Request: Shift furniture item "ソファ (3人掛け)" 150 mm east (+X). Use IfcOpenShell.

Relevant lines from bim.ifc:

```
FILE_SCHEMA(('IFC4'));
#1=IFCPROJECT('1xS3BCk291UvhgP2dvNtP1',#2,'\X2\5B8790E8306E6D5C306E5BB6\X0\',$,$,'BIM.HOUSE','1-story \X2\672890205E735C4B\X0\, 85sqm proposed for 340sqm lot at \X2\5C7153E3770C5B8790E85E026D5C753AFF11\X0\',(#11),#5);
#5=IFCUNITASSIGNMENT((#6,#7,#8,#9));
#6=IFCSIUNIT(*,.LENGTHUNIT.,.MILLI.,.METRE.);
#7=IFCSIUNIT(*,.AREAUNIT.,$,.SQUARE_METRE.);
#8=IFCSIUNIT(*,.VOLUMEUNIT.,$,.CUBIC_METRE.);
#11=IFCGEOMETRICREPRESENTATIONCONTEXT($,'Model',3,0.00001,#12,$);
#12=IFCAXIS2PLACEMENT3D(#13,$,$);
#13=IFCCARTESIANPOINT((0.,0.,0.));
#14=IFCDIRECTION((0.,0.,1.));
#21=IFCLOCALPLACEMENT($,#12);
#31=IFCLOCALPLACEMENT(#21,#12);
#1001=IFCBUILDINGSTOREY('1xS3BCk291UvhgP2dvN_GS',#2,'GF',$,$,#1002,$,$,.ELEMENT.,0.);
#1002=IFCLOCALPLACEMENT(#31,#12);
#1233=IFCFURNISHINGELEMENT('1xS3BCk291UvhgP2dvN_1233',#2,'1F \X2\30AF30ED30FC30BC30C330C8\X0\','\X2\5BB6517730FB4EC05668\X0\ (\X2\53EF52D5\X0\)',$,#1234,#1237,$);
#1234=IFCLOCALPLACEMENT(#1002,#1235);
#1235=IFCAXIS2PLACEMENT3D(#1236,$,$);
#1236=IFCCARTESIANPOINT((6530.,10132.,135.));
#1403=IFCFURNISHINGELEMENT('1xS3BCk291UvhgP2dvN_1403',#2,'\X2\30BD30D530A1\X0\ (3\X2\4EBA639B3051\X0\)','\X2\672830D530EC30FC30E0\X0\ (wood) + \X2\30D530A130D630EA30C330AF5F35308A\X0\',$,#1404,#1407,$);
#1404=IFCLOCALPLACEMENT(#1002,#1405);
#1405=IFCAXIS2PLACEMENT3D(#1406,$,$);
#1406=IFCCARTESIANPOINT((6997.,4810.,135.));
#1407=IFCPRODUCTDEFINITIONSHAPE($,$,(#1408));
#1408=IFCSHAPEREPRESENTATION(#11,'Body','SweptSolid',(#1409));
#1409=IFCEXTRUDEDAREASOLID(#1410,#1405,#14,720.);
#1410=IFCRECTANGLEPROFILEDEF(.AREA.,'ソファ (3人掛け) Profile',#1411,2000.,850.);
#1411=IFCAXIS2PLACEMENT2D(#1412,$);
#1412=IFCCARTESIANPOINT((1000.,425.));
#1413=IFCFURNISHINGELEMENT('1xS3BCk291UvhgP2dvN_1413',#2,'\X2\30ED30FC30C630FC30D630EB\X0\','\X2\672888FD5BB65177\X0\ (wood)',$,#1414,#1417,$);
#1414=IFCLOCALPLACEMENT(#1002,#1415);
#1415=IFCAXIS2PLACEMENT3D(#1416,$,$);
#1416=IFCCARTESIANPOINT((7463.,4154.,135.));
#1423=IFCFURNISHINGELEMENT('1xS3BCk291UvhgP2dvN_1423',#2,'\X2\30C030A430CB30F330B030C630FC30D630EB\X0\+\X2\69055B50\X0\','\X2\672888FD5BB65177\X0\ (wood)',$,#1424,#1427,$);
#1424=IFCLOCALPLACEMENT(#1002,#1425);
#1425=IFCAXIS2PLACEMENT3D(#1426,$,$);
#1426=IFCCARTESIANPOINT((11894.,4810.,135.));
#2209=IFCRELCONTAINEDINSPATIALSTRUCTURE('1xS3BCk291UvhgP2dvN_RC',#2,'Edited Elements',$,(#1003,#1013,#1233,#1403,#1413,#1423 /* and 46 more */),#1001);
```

```python
import ifcopenshell
import ifcopenshell.api.geometry
import ifcopenshell.util.placement
import ifcopenshell.util.unit

model = ifcopenshell.open("bim.ifc")
unit_scale = ifcopenshell.util.unit.calculate_unit_scale(model)

item = model.by_id(1403)
matrix = ifcopenshell.util.placement.get_local_placement(item.ObjectPlacement)
matrix[0, 3] += 0.15 / unit_scale
ifcopenshell.api.geometry.edit_object_placement(model, product=item, matrix=matrix, is_si=False)

print(ifcopenshell.util.placement.get_local_placement(item.ObjectPlacement).round(3) + 0.0)

model.write("bim_edited.ifc")
```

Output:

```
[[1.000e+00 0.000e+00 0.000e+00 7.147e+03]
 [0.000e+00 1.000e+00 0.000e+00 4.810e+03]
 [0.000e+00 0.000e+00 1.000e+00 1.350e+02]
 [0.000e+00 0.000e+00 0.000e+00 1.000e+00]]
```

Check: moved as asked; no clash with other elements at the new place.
